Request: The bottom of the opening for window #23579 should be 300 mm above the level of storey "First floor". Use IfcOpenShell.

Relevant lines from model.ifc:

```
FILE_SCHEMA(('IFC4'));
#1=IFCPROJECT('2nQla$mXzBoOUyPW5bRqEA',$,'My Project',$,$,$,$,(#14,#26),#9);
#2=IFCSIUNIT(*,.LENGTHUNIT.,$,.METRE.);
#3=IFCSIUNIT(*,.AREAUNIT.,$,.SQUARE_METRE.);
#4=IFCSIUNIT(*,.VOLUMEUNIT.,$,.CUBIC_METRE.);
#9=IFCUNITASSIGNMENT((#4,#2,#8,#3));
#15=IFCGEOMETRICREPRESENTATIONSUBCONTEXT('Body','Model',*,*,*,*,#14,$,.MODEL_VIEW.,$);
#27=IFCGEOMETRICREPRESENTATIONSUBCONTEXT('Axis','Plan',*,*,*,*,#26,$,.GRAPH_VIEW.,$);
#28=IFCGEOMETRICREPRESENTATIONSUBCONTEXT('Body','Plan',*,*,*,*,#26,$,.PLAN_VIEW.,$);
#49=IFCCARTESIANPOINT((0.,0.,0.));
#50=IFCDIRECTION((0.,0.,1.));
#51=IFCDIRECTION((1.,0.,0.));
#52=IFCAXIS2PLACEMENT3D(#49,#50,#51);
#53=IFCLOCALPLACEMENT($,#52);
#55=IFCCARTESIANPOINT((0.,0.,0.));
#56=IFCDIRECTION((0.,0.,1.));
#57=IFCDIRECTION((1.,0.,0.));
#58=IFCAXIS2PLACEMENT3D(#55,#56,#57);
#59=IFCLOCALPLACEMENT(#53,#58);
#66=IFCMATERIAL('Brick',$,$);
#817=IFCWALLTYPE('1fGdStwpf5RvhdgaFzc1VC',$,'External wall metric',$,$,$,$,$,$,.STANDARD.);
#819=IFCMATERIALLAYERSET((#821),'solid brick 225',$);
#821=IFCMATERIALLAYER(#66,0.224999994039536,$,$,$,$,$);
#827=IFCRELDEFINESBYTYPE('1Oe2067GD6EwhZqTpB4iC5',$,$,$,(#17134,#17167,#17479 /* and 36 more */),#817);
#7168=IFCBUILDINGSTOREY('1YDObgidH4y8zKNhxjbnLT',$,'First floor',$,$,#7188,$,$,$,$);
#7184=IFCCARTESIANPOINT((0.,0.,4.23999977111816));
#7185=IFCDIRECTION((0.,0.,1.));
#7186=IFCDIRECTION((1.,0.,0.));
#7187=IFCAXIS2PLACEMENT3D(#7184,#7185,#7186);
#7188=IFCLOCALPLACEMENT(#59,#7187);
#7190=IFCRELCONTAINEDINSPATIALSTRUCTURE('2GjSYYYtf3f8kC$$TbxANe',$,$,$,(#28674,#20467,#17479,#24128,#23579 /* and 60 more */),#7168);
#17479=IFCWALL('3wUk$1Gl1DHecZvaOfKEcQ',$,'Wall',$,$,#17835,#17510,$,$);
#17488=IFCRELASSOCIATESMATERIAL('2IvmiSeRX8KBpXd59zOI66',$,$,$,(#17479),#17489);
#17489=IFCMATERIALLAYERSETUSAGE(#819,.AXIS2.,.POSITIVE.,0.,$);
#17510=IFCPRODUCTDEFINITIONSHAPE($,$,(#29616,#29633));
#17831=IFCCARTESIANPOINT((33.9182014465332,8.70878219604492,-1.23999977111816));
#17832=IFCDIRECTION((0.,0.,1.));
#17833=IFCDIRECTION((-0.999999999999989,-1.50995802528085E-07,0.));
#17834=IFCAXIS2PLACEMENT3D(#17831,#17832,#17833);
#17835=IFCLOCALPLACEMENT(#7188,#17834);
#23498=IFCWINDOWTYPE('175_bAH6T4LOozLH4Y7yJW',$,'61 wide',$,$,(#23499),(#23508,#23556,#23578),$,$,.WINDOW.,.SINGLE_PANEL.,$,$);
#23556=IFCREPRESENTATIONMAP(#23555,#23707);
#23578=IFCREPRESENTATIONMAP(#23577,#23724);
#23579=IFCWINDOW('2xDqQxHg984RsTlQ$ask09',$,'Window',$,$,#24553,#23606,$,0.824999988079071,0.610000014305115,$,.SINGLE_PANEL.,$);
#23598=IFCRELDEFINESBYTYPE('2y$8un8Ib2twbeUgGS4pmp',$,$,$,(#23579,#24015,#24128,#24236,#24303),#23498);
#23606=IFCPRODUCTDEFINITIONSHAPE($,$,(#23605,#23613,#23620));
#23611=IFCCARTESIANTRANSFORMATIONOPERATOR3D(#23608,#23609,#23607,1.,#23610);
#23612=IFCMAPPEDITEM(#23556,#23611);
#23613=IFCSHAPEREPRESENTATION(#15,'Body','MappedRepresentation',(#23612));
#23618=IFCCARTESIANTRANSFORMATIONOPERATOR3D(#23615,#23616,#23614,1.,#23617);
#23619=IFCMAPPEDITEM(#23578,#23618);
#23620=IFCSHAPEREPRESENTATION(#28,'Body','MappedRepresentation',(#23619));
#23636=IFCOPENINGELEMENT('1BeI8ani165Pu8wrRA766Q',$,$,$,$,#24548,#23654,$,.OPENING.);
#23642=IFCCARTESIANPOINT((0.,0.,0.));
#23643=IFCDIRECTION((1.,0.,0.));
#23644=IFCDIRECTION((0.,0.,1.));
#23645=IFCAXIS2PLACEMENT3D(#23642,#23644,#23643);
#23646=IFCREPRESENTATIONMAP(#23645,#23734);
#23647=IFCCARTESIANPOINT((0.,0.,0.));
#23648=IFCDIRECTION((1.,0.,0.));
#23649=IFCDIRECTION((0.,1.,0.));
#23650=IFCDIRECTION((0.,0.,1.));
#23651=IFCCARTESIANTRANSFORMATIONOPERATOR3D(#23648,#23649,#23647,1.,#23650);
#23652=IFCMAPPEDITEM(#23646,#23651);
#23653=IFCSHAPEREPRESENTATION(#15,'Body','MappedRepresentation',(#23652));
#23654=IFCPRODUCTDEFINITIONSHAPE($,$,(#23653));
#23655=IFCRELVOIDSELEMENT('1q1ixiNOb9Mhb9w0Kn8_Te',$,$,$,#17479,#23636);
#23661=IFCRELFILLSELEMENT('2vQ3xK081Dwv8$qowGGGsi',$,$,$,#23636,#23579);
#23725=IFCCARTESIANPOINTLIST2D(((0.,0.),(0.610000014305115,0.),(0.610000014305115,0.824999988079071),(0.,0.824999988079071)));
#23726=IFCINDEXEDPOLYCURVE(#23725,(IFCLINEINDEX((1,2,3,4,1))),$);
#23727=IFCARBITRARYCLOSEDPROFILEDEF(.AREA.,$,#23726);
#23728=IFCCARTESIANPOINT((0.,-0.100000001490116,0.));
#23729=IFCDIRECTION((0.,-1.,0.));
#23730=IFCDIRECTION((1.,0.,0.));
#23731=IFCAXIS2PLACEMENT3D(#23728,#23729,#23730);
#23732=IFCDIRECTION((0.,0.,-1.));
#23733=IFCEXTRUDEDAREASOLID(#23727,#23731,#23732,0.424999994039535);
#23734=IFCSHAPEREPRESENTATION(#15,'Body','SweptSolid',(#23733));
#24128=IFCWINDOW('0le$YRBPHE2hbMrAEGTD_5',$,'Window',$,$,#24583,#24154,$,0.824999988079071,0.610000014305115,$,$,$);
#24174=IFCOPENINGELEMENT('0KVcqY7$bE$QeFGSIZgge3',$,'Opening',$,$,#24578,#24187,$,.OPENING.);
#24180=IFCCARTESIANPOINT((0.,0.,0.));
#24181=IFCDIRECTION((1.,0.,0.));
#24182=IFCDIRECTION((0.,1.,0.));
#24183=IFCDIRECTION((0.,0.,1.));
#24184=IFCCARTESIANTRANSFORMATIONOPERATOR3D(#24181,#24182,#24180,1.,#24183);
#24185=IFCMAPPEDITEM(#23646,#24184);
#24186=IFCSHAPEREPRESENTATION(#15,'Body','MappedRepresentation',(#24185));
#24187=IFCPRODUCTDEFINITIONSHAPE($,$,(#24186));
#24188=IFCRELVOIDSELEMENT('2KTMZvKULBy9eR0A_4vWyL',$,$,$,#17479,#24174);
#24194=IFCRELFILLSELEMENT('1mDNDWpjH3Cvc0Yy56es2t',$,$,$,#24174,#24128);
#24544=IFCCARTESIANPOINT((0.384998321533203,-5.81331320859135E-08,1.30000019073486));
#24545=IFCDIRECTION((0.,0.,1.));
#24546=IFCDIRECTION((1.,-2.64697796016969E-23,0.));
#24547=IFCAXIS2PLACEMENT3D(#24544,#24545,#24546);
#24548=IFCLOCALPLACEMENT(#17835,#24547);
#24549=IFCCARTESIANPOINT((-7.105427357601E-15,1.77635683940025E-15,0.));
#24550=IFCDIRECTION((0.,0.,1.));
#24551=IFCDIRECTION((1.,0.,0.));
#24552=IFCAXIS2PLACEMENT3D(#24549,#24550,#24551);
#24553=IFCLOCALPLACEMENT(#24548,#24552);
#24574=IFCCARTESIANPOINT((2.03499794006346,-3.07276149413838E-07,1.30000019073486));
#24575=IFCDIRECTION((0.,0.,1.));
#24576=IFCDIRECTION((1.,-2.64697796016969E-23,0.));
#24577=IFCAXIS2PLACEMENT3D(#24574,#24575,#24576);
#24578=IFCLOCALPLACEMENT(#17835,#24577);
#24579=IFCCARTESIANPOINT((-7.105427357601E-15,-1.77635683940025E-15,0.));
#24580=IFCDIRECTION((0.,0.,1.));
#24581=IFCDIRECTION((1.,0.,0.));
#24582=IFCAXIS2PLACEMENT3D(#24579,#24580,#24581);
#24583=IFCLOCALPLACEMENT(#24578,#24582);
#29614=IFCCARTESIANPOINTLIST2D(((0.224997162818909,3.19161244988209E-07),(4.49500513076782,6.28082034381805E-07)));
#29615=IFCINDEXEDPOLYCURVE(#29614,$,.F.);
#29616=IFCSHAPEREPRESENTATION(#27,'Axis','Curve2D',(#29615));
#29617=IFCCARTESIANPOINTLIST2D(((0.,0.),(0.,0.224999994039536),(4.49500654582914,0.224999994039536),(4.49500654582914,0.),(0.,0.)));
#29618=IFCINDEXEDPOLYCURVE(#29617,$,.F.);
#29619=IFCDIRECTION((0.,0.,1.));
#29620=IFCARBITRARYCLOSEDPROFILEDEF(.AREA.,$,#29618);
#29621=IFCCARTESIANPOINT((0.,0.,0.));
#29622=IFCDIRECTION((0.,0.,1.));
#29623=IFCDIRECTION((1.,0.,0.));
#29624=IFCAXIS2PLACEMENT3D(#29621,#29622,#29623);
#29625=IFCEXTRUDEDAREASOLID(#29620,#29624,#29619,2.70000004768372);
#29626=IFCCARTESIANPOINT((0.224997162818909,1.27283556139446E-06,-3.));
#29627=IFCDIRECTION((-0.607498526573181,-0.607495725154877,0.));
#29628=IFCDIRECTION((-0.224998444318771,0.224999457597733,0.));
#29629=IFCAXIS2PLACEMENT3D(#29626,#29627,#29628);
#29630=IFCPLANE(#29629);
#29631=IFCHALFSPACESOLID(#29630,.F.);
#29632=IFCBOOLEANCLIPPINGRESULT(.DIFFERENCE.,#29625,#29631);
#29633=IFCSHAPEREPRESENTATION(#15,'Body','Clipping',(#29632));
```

```python
import numpy as np
import ifcopenshell
import ifcopenshell.api.geometry
import ifcopenshell.geom
import ifcopenshell.util.element
import ifcopenshell.util.placement
import ifcopenshell.util.shape
import ifcopenshell.util.unit

model = ifcopenshell.open("model.ifc")
unit_scale = ifcopenshell.util.unit.calculate_unit_scale(model)

window = model.by_id(23579)
opening = window.FillsVoids[0].RelatingOpeningElement
storey = ifcopenshell.util.element.get_container(window, ifc_class="IfcBuildingStorey")
level = ifcopenshell.util.placement.get_local_placement(storey.ObjectPlacement)[2, 3]

# The opening's origin need not be at the sill, so measure its lowest point.
shape = ifcopenshell.geom.create_shape(ifcopenshell.geom.settings(), opening)
bottom = ifcopenshell.util.shape.get_shape_bottom_elevation(shape, shape.geometry) / unit_scale
dz = level + 0.3 - bottom

shift = np.array([0.0, 0.0, dz])
# The window is placed relative to its opening, so it follows when the opening moves.
matrix = ifcopenshell.util.placement.get_local_placement(opening.ObjectPlacement)
matrix[:3, 3] += shift
ifcopenshell.api.geometry.edit_object_placement(
    model, product=opening, matrix=matrix, is_si=False, should_transform_children=True
)

print(f"moved by {dz * unit_scale:+.3f} m")

model.write("model_edited.ifc")
```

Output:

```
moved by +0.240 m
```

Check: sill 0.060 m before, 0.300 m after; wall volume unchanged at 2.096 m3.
